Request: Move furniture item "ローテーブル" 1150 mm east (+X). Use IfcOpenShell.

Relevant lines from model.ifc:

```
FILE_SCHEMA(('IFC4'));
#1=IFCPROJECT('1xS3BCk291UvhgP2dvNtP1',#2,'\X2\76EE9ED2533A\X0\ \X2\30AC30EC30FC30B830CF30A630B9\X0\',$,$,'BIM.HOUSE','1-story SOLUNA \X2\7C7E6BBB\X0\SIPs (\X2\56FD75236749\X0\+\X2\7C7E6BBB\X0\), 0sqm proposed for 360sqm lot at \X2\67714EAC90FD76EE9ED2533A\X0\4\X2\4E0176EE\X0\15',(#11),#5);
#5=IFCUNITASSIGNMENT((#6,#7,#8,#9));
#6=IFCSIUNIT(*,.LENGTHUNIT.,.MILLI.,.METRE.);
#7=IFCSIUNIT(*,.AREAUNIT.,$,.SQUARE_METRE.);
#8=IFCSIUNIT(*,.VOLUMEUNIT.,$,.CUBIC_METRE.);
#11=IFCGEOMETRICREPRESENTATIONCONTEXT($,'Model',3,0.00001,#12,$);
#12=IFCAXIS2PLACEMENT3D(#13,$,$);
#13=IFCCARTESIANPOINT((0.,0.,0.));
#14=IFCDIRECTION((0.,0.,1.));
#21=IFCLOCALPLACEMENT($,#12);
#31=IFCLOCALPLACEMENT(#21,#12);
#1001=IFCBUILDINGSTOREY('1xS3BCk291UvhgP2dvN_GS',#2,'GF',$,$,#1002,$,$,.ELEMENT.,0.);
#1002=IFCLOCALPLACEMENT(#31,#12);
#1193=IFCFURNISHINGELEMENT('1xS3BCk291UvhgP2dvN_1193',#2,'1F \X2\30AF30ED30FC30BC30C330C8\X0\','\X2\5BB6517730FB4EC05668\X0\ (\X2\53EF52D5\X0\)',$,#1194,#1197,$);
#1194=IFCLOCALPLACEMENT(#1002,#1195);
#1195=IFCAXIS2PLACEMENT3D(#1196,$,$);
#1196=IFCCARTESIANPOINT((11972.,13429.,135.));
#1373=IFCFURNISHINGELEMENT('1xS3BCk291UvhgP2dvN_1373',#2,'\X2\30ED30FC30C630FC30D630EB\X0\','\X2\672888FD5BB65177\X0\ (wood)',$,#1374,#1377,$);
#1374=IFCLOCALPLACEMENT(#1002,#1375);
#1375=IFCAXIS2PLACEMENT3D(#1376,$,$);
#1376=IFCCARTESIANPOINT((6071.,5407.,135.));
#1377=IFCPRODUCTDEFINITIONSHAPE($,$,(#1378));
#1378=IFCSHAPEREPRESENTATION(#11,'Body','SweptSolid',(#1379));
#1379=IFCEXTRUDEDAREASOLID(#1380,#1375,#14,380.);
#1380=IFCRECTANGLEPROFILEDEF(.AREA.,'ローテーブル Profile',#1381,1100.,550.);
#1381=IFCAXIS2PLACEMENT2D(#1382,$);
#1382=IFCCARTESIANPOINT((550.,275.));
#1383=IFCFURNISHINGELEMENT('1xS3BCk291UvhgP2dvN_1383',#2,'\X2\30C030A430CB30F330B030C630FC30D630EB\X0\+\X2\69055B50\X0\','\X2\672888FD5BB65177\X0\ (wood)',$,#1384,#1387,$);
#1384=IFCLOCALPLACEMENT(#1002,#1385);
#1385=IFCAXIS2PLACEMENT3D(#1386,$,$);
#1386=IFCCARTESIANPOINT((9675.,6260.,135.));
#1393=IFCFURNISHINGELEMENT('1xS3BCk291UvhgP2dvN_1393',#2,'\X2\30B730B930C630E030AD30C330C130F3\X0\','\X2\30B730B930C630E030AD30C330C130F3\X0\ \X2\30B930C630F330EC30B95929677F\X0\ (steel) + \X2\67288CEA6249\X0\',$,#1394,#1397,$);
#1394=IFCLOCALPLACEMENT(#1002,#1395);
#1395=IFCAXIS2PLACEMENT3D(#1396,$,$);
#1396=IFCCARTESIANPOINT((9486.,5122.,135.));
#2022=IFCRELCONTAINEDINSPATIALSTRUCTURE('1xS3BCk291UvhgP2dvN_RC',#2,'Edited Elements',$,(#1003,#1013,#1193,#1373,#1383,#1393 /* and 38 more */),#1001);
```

```python
import ifcopenshell
import ifcopenshell.api.geometry
import ifcopenshell.util.placement
import ifcopenshell.util.unit

model = ifcopenshell.open("model.ifc")
unit_scale = ifcopenshell.util.unit.calculate_unit_scale(model)

item = model.by_guid("1xS3BCk291UvhgP2dvN_1373")
matrix = ifcopenshell.util.placement.get_local_placement(item.ObjectPlacement)
matrix[0, 3] += 1.15 / unit_scale
ifcopenshell.api.geometry.edit_object_placement(model, product=item, matrix=matrix, is_si=False)

print(ifcopenshell.util.placement.get_local_placement(item.ObjectPlacement).round(3) + 0.0)

model.write("model_edited.ifc")
```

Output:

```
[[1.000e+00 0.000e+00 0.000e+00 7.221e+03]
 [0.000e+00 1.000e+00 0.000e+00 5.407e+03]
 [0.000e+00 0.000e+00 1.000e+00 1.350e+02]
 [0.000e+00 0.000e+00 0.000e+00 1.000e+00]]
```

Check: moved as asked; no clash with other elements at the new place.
